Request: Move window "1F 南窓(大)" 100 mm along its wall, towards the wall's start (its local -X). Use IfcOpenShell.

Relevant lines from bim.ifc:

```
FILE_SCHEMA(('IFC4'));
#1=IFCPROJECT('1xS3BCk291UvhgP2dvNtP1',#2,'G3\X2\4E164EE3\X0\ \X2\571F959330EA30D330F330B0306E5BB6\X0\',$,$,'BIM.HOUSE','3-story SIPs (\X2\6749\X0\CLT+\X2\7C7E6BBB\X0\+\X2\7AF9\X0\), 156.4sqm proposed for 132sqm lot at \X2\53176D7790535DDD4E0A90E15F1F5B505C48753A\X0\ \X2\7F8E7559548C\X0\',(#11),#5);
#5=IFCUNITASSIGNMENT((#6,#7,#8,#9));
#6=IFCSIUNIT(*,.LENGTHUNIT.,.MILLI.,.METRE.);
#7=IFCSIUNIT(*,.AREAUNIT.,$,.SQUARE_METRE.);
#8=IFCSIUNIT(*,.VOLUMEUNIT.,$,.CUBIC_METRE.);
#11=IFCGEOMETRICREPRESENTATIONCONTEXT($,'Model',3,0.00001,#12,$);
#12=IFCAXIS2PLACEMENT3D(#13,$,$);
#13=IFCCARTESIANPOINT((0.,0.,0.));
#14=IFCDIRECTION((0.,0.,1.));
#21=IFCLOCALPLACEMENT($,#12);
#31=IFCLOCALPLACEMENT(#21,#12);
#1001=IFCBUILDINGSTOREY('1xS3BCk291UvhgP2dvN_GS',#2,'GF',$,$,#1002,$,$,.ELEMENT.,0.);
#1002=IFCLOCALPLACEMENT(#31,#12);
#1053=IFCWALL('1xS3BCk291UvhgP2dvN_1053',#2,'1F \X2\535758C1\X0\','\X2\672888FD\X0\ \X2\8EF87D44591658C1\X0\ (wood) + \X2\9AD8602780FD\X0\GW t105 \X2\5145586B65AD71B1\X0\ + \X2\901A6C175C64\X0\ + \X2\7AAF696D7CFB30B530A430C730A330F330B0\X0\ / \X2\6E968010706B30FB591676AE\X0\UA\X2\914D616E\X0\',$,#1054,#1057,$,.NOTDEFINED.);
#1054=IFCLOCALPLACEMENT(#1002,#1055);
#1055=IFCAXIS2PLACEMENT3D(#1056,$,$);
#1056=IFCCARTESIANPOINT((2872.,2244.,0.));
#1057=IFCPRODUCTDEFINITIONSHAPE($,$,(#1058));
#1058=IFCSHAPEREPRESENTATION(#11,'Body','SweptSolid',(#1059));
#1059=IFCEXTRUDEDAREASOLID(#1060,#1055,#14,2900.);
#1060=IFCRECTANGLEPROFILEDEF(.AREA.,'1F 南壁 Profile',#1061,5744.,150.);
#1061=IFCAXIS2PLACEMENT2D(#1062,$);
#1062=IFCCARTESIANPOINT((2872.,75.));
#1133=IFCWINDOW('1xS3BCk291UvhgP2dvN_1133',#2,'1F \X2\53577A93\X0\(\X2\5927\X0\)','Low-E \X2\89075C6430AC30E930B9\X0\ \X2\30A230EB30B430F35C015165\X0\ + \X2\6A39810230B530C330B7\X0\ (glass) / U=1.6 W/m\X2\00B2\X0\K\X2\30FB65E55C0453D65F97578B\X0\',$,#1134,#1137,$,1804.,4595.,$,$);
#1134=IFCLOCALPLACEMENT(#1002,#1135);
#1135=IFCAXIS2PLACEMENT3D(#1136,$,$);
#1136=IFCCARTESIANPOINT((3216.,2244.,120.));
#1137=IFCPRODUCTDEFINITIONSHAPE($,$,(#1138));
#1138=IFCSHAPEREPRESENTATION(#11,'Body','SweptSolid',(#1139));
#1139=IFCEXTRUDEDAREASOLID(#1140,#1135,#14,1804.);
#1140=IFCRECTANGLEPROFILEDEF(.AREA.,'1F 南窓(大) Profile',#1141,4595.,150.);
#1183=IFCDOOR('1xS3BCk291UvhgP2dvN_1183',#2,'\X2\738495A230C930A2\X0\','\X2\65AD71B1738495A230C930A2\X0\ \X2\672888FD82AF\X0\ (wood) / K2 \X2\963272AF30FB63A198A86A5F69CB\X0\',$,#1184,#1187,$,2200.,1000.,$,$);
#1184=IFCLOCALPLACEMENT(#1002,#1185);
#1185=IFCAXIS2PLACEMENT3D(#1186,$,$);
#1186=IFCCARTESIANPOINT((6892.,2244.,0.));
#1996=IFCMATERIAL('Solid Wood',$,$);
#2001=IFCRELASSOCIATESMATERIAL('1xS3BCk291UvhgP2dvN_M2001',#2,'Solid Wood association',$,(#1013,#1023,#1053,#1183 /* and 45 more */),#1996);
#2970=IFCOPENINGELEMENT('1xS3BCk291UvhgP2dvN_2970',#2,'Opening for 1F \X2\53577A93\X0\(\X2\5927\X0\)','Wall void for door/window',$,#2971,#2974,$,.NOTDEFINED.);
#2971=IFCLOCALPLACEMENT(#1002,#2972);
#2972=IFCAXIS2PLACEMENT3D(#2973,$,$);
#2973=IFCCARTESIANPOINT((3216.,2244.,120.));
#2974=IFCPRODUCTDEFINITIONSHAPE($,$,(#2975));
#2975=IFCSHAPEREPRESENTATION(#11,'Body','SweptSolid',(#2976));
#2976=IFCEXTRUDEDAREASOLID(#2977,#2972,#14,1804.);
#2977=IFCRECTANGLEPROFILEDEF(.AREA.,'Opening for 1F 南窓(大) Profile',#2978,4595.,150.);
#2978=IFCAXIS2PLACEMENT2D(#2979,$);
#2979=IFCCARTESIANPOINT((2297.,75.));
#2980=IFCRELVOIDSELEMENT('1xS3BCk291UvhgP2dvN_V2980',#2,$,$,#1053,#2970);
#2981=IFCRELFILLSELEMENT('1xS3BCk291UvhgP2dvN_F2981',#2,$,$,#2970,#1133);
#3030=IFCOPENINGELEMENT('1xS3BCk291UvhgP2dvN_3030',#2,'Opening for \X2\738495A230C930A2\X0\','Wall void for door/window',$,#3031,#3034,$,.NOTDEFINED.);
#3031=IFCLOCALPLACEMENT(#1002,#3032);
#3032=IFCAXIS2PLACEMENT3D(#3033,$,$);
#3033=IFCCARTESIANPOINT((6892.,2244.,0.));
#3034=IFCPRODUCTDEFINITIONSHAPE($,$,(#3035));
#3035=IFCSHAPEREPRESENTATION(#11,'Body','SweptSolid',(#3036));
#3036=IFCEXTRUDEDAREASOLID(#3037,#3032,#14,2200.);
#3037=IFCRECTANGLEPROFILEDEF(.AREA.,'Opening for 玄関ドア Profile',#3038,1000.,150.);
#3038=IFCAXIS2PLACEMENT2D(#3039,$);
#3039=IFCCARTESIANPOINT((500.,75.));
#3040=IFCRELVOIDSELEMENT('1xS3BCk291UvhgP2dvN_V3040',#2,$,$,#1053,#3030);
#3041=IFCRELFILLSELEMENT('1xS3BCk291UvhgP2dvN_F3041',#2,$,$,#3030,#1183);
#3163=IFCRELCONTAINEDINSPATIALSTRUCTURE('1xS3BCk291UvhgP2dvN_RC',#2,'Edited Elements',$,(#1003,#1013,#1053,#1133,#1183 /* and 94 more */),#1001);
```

```python
import ifcopenshell
import ifcopenshell.api.geometry
import ifcopenshell.util.placement

model = ifcopenshell.open("bim.ifc")

window = model.by_guid("1xS3BCk291UvhgP2dvN_1133")
opening = window.FillsVoids[0].RelatingOpeningElement
wall = opening.VoidsElements[0].RelatingBuildingElement

wall_matrix = ifcopenshell.util.placement.get_local_placement(wall.ObjectPlacement)
shift = wall_matrix[:3, 0] * -100.0
before = ifcopenshell.util.placement.get_local_placement(window.ObjectPlacement)[:3, 3].copy()

# The window is not placed relative to its opening, so move both.
for product in (opening, window):
    matrix = ifcopenshell.util.placement.get_local_placement(product.ObjectPlacement)
    matrix[:3, 3] += shift
    ifcopenshell.api.geometry.edit_object_placement(model, product=product, matrix=matrix, is_si=False)

after = ifcopenshell.util.placement.get_local_placement(window.ObjectPlacement)[:3, 3]
print("window moved by", (after - before).round(3) + 0.0)

model.write("bim_rev.ifc")
```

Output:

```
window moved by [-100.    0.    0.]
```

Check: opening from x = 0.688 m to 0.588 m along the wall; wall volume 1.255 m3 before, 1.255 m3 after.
